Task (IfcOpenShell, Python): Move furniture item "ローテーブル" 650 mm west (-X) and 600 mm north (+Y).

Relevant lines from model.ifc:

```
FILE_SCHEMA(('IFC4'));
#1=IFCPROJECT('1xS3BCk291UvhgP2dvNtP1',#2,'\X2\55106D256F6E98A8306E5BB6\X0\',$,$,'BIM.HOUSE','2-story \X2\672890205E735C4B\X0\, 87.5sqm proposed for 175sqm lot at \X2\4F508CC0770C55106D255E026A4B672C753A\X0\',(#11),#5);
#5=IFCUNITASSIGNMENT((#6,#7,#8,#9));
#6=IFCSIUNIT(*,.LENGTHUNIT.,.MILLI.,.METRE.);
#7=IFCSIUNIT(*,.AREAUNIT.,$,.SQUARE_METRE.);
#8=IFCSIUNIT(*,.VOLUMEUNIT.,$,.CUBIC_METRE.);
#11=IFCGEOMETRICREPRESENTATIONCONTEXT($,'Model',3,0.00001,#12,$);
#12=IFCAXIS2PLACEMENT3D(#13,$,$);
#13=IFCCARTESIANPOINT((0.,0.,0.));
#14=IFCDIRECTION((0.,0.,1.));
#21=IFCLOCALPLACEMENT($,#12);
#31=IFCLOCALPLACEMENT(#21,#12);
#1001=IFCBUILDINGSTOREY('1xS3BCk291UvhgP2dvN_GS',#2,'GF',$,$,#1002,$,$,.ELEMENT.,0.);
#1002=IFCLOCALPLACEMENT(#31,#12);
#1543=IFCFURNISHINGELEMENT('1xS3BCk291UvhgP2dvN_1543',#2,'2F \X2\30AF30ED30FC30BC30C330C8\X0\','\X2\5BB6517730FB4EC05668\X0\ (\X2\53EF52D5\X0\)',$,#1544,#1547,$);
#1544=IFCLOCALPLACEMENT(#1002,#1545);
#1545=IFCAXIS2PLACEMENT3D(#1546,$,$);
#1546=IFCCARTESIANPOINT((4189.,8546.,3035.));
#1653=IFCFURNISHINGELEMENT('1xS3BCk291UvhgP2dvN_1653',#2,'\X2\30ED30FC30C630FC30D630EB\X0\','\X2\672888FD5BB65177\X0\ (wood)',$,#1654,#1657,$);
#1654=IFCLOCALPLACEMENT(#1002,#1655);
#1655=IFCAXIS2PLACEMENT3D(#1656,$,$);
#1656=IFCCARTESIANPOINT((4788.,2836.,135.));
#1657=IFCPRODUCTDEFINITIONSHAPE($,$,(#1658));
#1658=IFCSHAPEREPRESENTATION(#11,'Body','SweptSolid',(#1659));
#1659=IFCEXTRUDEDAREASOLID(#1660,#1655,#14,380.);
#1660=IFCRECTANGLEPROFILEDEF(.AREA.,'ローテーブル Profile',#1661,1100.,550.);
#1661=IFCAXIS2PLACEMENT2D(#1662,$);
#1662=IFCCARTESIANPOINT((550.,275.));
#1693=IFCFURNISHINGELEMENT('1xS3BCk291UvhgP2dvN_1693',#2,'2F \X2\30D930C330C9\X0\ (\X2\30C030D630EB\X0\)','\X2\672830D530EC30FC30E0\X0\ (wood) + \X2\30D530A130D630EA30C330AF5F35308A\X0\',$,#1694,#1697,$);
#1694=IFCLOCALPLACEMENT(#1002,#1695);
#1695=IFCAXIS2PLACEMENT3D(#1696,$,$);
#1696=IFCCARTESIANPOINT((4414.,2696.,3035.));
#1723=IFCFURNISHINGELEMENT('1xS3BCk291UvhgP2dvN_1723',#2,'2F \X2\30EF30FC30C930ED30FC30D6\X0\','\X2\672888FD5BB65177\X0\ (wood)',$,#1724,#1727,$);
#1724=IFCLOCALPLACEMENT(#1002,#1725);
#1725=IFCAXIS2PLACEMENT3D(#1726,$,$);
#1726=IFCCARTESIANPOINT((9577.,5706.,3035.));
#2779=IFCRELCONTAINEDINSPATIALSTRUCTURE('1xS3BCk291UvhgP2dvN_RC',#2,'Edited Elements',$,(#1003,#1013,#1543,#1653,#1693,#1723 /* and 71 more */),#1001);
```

```python
import ifcopenshell
import ifcopenshell.api.geometry
import ifcopenshell.util.placement
import ifcopenshell.util.unit

model = ifcopenshell.open("model.ifc")
unit_scale = ifcopenshell.util.unit.calculate_unit_scale(model)

item = model.by_guid("1xS3BCk291UvhgP2dvN_1653")
matrix = ifcopenshell.util.placement.get_local_placement(item.ObjectPlacement)
matrix[0, 3] -= 0.65 / unit_scale
matrix[1, 3] += 0.6 / unit_scale
ifcopenshell.api.geometry.edit_object_placement(model, product=item, matrix=matrix, is_si=False)

print(ifcopenshell.util.placement.get_local_placement(item.ObjectPlacement).round(3) + 0.0)

model.write("model_edited.ifc")
```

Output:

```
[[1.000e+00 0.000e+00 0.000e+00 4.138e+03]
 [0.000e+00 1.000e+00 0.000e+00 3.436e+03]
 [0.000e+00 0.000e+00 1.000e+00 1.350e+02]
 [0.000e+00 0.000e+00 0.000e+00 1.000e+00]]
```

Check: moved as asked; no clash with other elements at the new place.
